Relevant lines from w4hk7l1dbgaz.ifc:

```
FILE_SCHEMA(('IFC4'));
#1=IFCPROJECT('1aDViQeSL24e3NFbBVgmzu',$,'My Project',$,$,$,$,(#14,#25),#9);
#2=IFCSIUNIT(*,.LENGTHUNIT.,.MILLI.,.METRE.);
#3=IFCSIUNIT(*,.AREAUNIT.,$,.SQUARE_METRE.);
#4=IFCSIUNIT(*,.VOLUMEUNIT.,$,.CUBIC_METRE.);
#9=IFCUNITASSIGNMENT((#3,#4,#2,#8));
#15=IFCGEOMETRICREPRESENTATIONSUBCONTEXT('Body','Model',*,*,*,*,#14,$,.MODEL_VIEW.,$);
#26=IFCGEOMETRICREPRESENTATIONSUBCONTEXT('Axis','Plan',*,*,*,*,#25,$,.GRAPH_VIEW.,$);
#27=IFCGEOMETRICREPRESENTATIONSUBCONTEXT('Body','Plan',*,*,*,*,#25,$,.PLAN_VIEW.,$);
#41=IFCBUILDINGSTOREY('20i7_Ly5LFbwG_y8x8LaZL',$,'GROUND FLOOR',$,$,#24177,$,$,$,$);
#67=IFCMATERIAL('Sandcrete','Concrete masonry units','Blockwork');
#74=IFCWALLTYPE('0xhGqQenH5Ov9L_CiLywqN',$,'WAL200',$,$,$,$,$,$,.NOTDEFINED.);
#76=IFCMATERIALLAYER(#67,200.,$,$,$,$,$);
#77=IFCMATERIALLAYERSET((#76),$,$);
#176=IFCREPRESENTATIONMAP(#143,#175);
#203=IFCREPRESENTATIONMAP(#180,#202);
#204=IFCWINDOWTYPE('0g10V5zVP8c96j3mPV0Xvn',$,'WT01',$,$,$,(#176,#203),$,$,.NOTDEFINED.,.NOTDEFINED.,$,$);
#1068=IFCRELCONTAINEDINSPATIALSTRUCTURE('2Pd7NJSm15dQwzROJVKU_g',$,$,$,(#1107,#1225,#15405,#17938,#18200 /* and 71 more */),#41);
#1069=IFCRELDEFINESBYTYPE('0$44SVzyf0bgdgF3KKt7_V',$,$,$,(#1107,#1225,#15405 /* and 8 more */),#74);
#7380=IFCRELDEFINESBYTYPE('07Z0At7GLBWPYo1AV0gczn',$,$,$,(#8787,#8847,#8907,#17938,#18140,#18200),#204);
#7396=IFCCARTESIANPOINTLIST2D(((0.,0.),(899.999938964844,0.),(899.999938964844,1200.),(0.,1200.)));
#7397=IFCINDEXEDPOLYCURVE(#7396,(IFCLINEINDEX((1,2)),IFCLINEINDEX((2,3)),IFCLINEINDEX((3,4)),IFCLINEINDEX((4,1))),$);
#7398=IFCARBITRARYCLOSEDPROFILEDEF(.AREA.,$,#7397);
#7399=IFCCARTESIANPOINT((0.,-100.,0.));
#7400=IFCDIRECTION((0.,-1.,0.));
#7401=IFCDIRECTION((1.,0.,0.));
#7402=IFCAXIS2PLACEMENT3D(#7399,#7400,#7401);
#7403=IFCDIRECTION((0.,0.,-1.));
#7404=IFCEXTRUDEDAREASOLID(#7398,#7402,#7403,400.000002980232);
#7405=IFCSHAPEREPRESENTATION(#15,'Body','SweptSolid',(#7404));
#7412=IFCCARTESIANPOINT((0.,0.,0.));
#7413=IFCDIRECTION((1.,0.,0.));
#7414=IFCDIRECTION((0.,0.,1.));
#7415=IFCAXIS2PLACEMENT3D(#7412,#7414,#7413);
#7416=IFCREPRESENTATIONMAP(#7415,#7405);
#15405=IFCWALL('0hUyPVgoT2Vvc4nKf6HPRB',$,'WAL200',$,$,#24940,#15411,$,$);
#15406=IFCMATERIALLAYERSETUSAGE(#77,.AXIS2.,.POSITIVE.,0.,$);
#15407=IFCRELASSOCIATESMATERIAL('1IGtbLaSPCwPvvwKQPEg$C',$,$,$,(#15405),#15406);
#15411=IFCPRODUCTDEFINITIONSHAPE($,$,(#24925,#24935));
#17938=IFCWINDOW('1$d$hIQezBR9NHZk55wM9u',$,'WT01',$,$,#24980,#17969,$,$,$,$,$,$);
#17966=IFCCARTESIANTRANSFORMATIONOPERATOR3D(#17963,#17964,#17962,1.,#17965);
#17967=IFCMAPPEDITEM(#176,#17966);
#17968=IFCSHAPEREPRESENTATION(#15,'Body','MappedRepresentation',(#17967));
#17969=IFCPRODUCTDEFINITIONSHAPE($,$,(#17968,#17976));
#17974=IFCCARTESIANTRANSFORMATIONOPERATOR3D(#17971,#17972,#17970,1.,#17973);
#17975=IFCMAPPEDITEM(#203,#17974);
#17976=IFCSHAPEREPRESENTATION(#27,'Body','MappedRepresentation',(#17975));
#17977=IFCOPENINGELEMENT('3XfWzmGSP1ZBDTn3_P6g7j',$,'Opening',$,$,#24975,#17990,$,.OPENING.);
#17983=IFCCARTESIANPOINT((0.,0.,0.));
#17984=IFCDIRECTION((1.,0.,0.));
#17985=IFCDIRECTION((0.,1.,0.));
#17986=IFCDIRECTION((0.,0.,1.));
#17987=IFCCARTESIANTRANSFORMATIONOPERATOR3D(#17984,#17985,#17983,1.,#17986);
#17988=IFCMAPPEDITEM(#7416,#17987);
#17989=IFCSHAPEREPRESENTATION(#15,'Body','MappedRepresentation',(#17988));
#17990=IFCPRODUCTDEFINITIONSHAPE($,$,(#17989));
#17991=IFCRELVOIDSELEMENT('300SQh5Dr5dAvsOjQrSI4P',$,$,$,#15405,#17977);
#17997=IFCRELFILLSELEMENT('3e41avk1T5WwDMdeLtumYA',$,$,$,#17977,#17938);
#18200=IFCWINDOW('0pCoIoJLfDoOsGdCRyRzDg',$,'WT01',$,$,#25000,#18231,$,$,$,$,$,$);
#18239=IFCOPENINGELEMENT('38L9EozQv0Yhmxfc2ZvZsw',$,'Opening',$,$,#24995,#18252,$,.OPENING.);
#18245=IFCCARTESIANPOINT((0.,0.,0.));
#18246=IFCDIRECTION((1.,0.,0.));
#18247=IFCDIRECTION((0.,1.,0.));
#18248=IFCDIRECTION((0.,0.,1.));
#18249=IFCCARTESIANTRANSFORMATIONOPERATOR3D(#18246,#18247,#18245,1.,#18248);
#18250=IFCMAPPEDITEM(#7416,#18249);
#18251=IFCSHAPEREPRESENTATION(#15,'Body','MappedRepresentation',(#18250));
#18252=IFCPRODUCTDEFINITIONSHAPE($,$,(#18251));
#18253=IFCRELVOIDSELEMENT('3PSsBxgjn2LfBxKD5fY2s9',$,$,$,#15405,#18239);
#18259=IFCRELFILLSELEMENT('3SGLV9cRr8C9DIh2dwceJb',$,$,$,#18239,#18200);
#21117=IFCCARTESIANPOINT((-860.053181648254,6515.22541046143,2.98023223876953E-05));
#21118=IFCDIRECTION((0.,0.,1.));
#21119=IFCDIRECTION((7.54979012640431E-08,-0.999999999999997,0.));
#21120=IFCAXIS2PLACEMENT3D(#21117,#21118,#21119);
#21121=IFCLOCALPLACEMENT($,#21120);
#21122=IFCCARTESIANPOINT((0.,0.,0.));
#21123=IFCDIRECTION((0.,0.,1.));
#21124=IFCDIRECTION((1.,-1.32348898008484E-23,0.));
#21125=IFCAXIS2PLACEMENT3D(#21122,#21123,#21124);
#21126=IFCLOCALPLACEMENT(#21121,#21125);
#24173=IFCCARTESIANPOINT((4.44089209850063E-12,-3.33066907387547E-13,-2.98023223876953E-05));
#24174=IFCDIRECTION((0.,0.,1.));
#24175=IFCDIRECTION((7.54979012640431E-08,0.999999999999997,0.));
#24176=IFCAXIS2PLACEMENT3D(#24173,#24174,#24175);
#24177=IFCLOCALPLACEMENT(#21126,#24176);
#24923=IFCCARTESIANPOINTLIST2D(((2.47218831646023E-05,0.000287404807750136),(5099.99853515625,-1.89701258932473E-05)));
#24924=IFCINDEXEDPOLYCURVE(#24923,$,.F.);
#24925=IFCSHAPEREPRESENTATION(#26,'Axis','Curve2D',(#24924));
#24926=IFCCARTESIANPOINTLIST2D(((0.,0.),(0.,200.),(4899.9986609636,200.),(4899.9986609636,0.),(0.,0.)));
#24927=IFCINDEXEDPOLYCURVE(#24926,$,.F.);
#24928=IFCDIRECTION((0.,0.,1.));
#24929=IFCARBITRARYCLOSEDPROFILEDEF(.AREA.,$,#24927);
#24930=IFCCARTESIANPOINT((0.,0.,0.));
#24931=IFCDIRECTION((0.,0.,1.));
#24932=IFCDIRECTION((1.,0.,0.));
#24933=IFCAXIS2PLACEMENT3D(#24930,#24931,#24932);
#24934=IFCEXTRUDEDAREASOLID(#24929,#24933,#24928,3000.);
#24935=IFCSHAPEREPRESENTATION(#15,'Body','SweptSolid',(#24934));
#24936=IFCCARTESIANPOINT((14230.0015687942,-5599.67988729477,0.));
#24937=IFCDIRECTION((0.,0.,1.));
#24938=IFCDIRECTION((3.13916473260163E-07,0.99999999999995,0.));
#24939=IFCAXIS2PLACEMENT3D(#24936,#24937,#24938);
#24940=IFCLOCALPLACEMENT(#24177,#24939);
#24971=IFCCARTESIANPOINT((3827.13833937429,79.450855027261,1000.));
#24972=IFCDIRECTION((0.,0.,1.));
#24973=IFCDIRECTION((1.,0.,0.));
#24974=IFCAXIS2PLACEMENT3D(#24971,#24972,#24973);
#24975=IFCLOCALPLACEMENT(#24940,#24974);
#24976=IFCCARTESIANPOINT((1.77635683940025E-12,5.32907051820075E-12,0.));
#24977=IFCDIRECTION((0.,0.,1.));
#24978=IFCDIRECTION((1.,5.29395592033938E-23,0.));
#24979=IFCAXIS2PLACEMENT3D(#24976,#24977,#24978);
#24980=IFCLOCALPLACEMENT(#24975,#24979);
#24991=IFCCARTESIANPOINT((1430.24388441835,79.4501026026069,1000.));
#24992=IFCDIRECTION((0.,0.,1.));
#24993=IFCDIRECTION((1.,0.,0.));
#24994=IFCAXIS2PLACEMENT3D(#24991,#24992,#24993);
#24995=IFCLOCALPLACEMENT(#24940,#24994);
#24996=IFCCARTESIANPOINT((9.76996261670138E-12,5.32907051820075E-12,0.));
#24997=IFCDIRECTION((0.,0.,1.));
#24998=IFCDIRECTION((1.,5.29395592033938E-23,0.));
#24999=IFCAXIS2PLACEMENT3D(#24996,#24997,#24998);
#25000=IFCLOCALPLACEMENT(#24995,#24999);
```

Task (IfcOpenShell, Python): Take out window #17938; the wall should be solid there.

```python
import ifcopenshell
import ifcopenshell.api.feature
import ifcopenshell.api.root
import ifcopenshell.geom
import ifcopenshell.util.shape

model = ifcopenshell.open("w4hk7l1dbgaz.ifc")
settings = ifcopenshell.geom.settings()


def volume(element):
    """Net volume in cubic metres, openings subtracted."""
    shape = ifcopenshell.geom.create_shape(settings, element)
    return ifcopenshell.util.shape.get_volume(shape.geometry)


window = model.by_guid("1$d$hIQezBR9NHZk55wM9u")
opening = window.FillsVoids[0].RelatingOpeningElement
wall = opening.VoidsElements[0].RelatingBuildingElement
before = volume(wall)

ifcopenshell.api.root.remove_product(model, product=window)
ifcopenshell.api.feature.remove_feature(model, feature=opening)

after = volume(wall)

print(f"wall volume {before:.3f} -> {after:.3f} m3")

model.write("w4hk7l1dbgaz-out.ifc")
```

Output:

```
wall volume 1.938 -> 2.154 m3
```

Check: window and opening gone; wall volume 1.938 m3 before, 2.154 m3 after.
